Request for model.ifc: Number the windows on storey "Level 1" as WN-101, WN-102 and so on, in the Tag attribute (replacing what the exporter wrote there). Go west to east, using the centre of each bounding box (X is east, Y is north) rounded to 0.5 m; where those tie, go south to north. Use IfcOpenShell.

First a look at what the model holds.

```python
import ifcopenshell
import ifcopenshell.util.element
import ifcopenshell.util.placement

model = ifcopenshell.open("model.ifc")
print(model.schema)
storey = next(s for s in model.by_type("IfcBuildingStorey") if s.Name == "Level 1")
windows = [e for e in ifcopenshell.util.element.get_decomposition(storey) if e.is_a("IfcWindow")]
for e in sorted(windows, key=lambda e: e.id()):
    origin = ifcopenshell.util.placement.get_local_placement(e.ObjectPlacement)[:3, 3]
    print(e.id(), e.Tag, e.Name, origin.round(2) + 0.0, sep=" | ")
```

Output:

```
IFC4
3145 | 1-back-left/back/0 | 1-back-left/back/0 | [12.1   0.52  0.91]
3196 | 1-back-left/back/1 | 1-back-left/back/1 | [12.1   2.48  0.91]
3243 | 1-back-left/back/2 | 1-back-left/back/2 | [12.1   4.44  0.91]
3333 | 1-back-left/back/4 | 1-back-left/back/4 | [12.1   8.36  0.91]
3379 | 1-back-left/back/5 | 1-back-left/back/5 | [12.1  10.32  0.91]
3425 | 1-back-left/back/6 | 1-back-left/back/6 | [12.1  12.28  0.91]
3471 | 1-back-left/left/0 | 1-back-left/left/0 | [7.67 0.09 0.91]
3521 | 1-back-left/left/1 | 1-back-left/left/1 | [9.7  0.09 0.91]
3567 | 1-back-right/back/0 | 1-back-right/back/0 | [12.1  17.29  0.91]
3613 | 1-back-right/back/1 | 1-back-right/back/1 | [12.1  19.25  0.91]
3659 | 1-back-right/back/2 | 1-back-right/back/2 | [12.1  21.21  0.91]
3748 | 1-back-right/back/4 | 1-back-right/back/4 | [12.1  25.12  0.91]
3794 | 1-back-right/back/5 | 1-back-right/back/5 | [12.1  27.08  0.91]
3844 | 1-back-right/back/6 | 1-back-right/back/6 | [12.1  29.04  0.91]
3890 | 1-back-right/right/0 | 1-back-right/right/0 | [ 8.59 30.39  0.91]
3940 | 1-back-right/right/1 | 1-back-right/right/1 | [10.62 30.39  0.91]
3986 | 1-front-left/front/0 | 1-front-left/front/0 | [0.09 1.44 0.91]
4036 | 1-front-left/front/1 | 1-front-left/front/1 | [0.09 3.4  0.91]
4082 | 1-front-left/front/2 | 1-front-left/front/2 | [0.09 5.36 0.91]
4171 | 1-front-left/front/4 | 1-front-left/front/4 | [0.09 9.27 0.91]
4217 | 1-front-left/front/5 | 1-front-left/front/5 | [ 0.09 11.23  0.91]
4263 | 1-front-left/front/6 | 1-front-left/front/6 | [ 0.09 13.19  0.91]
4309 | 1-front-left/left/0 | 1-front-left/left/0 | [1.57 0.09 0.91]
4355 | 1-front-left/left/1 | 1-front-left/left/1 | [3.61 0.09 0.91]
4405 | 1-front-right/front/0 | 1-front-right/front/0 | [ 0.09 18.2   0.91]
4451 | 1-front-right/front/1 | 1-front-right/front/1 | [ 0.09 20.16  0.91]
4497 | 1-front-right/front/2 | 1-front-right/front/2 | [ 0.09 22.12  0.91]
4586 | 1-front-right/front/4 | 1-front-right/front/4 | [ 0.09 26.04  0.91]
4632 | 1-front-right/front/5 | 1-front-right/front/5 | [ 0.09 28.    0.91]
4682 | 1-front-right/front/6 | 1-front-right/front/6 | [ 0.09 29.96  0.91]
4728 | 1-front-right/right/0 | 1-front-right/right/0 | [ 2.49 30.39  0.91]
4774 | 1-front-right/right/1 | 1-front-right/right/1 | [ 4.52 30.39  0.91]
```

```python
import ifcopenshell
import ifcopenshell.geom
import ifcopenshell.util.element
import ifcopenshell.util.shape

model = ifcopenshell.open("model.ifc")
settings = ifcopenshell.geom.settings()
settings.set("use-world-coords", True)


def centre(element):
    shape = ifcopenshell.geom.create_shape(settings, element)
    return ifcopenshell.util.shape.get_bbox_centroid(shape.geometry)


storey = next(s for s in model.by_type("IfcBuildingStorey") if s.Name == "Level 1")
windows = [e for e in ifcopenshell.util.element.get_decomposition(storey) if e.is_a("IfcWindow")]

# Insertion points can sit at a corner or the storey origin, so sort by the geometry (in metres).
centres = {e: centre(e) for e in windows}
windows.sort(key=lambda e: (round(centres[e][0] / 0.5), centres[e][1]))

for i, e in enumerate(windows, start=1):
    number = f"WN-1{i:02d}"
    e.Tag = number
    print(e.id(), number)

model.write("model_rev.ifc")
```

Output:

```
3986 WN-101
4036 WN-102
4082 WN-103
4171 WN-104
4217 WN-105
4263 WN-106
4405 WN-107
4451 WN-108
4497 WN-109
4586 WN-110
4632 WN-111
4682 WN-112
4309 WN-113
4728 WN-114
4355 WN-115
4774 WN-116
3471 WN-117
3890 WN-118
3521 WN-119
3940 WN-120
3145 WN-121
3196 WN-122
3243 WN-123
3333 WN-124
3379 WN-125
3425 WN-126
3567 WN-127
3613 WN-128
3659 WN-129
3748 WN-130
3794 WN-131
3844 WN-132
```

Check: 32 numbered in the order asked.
